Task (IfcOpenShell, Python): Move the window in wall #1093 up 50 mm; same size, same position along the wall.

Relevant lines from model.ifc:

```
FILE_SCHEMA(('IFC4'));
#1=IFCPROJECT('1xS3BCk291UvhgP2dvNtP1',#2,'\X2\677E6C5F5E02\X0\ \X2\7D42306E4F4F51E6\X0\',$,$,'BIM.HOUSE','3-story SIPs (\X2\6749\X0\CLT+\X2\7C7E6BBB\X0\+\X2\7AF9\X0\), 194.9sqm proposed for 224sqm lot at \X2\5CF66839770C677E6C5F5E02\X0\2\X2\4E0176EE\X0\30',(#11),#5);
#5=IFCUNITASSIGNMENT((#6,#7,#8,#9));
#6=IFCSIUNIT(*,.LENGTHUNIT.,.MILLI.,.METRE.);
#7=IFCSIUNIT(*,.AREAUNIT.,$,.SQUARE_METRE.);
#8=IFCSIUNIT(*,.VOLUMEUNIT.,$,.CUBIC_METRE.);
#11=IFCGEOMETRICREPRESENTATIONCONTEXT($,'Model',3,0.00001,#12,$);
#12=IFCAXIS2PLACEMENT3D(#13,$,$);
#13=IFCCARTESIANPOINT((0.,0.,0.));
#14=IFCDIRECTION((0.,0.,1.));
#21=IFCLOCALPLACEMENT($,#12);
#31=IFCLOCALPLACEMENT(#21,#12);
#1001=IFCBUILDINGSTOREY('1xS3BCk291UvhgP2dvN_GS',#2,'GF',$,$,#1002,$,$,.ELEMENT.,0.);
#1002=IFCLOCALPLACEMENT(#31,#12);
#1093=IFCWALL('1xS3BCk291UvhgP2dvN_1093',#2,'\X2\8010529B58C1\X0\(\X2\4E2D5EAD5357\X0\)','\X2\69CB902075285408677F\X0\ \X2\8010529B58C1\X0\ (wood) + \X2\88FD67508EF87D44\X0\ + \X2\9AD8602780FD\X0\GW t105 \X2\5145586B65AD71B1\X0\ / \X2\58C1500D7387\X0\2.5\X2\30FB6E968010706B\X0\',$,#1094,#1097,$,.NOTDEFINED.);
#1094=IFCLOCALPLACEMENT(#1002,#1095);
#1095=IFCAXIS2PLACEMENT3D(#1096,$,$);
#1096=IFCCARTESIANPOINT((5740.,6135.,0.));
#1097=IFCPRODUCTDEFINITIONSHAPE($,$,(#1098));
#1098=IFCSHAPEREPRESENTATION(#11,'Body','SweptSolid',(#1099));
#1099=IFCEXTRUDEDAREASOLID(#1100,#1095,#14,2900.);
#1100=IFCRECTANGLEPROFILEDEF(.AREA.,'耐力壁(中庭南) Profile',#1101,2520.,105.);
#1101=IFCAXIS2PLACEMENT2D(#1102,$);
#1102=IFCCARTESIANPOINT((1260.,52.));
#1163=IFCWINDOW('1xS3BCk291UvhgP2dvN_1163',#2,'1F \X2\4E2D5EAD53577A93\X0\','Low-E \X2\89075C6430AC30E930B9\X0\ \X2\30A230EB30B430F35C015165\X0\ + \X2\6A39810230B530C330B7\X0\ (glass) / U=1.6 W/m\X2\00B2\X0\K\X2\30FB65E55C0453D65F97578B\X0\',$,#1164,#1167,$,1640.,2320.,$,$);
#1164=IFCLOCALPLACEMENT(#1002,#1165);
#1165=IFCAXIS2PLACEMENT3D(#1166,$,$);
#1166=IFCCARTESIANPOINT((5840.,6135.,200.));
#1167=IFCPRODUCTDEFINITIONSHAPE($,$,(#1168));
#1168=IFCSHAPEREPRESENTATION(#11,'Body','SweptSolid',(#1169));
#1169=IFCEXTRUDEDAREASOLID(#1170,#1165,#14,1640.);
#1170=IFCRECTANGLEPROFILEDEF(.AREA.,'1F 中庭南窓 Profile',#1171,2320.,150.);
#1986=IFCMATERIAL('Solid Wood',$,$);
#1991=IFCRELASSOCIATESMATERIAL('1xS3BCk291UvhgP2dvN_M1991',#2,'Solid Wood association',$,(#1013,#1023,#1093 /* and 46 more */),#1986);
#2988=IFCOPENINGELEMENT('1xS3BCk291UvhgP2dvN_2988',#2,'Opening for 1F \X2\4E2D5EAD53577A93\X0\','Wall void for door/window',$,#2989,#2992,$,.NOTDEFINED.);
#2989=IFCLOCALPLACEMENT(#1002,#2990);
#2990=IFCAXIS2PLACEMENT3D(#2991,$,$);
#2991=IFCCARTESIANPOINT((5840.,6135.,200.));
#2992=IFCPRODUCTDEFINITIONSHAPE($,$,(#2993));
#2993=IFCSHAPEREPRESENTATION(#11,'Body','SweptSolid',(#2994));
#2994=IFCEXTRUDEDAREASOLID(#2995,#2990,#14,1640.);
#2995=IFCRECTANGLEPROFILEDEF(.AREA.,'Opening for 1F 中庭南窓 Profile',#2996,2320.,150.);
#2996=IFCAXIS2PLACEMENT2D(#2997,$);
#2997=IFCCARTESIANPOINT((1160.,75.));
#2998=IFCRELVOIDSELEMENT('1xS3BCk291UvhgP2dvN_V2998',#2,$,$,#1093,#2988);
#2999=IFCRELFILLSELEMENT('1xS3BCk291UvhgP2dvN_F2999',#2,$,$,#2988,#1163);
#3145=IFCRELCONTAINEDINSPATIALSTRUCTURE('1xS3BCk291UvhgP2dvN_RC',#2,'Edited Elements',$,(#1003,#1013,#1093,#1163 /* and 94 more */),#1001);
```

```python
import numpy as np
import ifcopenshell
import ifcopenshell.api.geometry
import ifcopenshell.util.placement
import ifcopenshell.util.unit

model = ifcopenshell.open("model.ifc")
unit_scale = ifcopenshell.util.unit.calculate_unit_scale(model)

window = model.by_guid("1xS3BCk291UvhgP2dvN_1163")
opening = window.FillsVoids[0].RelatingOpeningElement
dz = 50.0

shift = np.array([0.0, 0.0, dz])
# The window is not placed relative to its opening, so move both.
for product in (opening, window):
    matrix = ifcopenshell.util.placement.get_local_placement(product.ObjectPlacement)
    matrix[:3, 3] += shift
    ifcopenshell.api.geometry.edit_object_placement(model, product=product, matrix=matrix, is_si=False)

print(f"moved by {dz * unit_scale:+.3f} m")

model.write("model_edited.ifc")
```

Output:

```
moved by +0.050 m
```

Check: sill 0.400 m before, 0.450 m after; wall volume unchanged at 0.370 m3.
